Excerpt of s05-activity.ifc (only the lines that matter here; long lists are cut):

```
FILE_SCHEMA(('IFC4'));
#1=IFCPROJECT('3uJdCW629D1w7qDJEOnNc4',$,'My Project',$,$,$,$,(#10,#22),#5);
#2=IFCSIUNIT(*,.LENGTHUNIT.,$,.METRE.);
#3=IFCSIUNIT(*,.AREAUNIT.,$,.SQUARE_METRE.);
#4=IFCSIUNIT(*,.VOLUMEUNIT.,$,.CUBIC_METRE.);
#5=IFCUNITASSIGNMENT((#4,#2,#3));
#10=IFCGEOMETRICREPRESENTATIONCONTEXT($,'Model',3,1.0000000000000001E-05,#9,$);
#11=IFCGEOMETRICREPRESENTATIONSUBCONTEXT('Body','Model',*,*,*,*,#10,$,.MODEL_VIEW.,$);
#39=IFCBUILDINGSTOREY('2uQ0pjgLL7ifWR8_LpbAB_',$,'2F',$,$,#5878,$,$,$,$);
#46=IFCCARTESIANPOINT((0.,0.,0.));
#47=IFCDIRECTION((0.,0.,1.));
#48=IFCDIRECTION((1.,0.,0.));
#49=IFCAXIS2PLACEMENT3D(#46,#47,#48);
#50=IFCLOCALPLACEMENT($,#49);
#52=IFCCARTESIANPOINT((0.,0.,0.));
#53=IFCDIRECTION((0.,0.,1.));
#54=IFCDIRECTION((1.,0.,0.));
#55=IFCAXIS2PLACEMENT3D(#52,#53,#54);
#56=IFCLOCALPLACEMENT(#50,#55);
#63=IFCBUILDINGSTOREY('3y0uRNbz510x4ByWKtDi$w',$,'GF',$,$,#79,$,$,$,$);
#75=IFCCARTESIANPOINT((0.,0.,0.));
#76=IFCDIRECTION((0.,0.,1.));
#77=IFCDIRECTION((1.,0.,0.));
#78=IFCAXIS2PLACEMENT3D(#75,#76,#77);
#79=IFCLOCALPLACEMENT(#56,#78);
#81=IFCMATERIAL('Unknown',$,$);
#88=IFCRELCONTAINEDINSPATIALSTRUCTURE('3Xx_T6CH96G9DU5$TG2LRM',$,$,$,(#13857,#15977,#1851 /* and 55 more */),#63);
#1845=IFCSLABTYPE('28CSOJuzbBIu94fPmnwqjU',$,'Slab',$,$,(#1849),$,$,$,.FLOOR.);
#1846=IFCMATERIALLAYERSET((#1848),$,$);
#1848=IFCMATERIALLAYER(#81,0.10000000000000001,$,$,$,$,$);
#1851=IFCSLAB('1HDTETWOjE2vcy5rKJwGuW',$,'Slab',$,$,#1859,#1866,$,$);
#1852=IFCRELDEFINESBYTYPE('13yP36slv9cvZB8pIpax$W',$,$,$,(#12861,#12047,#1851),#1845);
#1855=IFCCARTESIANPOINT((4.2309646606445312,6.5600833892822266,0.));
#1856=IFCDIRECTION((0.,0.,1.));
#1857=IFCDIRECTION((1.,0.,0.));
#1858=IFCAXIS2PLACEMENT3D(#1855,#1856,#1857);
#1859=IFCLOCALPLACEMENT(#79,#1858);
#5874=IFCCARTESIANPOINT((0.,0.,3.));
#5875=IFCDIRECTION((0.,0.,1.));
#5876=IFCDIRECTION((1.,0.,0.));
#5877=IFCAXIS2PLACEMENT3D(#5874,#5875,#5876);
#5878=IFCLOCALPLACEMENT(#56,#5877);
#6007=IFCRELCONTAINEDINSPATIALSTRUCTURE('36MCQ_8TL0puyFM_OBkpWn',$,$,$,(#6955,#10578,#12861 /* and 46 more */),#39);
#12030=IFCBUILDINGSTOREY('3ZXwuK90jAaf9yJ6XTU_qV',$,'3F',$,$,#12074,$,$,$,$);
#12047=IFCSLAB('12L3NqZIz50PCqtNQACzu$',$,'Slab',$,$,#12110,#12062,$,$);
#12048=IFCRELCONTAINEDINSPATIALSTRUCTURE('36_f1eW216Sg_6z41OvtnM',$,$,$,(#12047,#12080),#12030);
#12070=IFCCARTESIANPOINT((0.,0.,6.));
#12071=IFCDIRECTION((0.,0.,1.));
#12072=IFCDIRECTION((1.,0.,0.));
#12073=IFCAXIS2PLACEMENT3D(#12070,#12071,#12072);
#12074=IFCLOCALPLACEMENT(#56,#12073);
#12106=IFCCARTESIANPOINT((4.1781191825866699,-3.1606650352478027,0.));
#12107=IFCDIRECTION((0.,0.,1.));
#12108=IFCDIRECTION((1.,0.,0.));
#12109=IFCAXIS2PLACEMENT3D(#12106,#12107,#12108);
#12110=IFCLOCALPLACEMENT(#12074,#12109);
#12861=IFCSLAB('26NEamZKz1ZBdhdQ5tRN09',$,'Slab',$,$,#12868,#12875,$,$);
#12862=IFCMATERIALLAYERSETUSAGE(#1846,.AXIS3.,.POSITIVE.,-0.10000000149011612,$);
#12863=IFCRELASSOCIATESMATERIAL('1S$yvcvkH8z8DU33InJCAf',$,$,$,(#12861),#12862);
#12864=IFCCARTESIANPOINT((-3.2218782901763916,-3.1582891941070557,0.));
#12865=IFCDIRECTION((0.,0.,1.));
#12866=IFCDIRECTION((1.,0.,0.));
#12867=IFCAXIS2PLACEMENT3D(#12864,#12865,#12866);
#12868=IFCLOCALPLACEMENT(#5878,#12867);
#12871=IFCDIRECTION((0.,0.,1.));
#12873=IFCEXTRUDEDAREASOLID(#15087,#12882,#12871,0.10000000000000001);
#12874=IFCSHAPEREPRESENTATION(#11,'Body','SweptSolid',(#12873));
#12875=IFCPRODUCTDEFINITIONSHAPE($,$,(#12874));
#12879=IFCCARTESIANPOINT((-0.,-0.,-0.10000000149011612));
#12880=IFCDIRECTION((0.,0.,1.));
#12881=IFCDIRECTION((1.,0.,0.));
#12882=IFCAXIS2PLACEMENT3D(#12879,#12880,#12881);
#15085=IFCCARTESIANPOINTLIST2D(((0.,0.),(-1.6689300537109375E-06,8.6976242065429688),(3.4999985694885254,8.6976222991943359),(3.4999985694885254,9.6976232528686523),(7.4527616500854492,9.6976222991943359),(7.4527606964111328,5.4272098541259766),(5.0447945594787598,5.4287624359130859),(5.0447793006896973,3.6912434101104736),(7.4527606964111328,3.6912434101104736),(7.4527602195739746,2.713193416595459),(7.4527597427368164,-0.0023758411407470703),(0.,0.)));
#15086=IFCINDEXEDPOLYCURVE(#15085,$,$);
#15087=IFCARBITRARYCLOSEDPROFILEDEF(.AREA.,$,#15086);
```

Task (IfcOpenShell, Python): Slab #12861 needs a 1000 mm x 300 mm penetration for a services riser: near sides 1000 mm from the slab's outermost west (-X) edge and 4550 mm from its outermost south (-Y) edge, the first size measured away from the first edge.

```python
import numpy as np
import ifcopenshell
import ifcopenshell.api.feature
import ifcopenshell.api.geometry
import ifcopenshell.api.root
import ifcopenshell.geom
import ifcopenshell.util.placement
import ifcopenshell.util.representation
import ifcopenshell.util.shape
import ifcopenshell.util.unit

model = ifcopenshell.open("s05-activity.ifc")
unit_scale = ifcopenshell.util.unit.calculate_unit_scale(model)
settings = ifcopenshell.geom.settings()


def volume(element):
    """Net volume in cubic metres, openings subtracted."""
    shape = ifcopenshell.geom.create_shape(settings, element)
    return ifcopenshell.util.shape.get_volume(shape.geometry)


slab = model.by_guid("26NEamZKz1ZBdhdQ5tRN09")
before = volume(slab)

# Extent in the slab's own axes, in metres. The edges named are its -X and -Y sides.
slab_shape = ifcopenshell.geom.create_shape(settings, slab)
vertices = ifcopenshell.util.shape.get_vertices(slab_shape.geometry)
x_min, y_min, bottom = vertices.min(axis=0)
top = vertices[:, 2].max()

opening = ifcopenshell.api.root.create_entity(model, ifc_class="IfcOpeningElement", name="Services riser opening", predefined_type="OPENING")
context = ifcopenshell.util.representation.get_context(model, "Model", "Body", "MODEL_VIEW")
width, depth = 1, 0.3
outline = [(0.0, 0.0), (width, 0.0), (width, depth), (0.0, depth), (0.0, 0.0)]
# Overshoot both faces by 50 mm so the cut is clean.
shape = ifcopenshell.api.geometry.add_slab_representation(
    model, context=context, depth=top - bottom + 0.1, polyline=outline
)
ifcopenshell.api.geometry.assign_representation(model, product=opening, representation=shape)

matrix = ifcopenshell.util.placement.get_local_placement(slab.ObjectPlacement)
matrix[:, 3] = matrix @ np.append(np.array([x_min + 1, y_min + 4.55, bottom - 0.05]) / unit_scale, 1.0)
ifcopenshell.api.geometry.edit_object_placement(model, product=opening, matrix=matrix, is_si=False)
ifcopenshell.api.feature.add_feature(model, feature=opening, element=slab)

after = volume(slab)

print(f"slab volume {before:.3f} -> {after:.3f} m3")

model.write("s05-activity_v2.ifc")
```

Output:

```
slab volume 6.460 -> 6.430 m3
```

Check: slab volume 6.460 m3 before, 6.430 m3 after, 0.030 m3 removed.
